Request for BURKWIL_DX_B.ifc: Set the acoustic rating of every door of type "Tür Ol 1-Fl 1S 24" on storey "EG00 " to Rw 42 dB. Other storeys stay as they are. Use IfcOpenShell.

First a look at what the model holds.

```python
import ifcopenshell
import ifcopenshell.util.element

model = ifcopenshell.open("BURKWIL_DX_B.ifc")
print(model.schema)
storey = next(s for s in model.by_type("IfcBuildingStorey") if s.Name == "EG00 ")
doors = [e for e in ifcopenshell.util.element.get_decomposition(storey) if e.is_a("IfcDoor")]
seen = {}
for e in doors:
    element_type = ifcopenshell.util.element.get_type(e)
    key = (element_type.Name if element_type != e and element_type else None, ifcopenshell.util.element.get_pset(e, "Pset_DoorCommon", "AcousticRating"))
    seen[key] = seen.get(key, 0) + 1
for (name, value), count in sorted(seen.items(), key=str):
    print(count, "x", name, "|", value)
```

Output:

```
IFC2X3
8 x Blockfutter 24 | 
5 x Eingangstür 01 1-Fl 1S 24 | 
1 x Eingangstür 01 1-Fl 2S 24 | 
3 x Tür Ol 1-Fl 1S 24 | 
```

```python
import ifcopenshell
import ifcopenshell.api.pset
import ifcopenshell.util.element

model = ifcopenshell.open("BURKWIL_DX_B.ifc")

storey = next(s for s in model.by_type("IfcBuildingStorey") if s.Name == "EG00 ")
doors = [e for e in ifcopenshell.util.element.get_decomposition(storey) if e.is_a("IfcDoor")]

count = 0
for e in doors:
    element_type = ifcopenshell.util.element.get_type(e)
    if element_type in (None, e) or element_type.Name != "Tür Ol 1-Fl 1S 24":
        continue
    # add_pset returns the element's existing set when there is one.
    pset = ifcopenshell.api.pset.add_pset(model, product=e, name="Pset_DoorCommon")
    ifcopenshell.api.pset.edit_pset(model, pset=pset, properties={"AcousticRating": "Rw 42 dB"})
    count += 1

print(count, "doors updated")

model.write("BURKWIL_DX_B_updated.ifc")
```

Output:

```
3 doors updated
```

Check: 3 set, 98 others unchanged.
